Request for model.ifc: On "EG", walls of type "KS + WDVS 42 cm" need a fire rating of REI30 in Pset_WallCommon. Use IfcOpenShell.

First a look at what the model holds.

```python
import ifcopenshell
import ifcopenshell.util.element

model = ifcopenshell.open("model.ifc")
print(model.schema)
storey = next(s for s in model.by_type("IfcBuildingStorey") if s.Name == "EG")
walls = [e for e in ifcopenshell.util.element.get_decomposition(storey) if e.is_a("IfcWall")]
seen = {}
for e in walls:
    element_type = ifcopenshell.util.element.get_type(e)
    key = (element_type.Name if element_type != e and element_type else None, ifcopenshell.util.element.get_pset(e, "Pset_WallCommon", "FireRating"))
    seen[key] = seen.get(key, 0) + 1
for (name, value), count in sorted(seen.items(), key=str):
    print(count, "x", name, "|", value)
```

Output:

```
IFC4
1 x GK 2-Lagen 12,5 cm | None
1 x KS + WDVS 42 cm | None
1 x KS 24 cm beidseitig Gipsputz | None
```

```python
import ifcopenshell
import ifcopenshell.api.pset
import ifcopenshell.util.element

model = ifcopenshell.open("model.ifc")

storey = next(s for s in model.by_type("IfcBuildingStorey") if s.Name == "EG")
walls = [e for e in ifcopenshell.util.element.get_decomposition(storey) if e.is_a("IfcWall")]

count = 0
for e in walls:
    element_type = ifcopenshell.util.element.get_type(e)
    if element_type in (None, e) or element_type.Name != "KS + WDVS 42 cm":
        continue
    # add_pset returns the element's existing set when there is one.
    pset = ifcopenshell.api.pset.add_pset(model, product=e, name="Pset_WallCommon")
    ifcopenshell.api.pset.edit_pset(model, pset=pset, properties={"FireRating": "REI30"})
    count += 1

print(count, "walls updated")

model.write("model_edited.ifc")
```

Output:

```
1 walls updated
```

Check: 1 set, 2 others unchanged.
